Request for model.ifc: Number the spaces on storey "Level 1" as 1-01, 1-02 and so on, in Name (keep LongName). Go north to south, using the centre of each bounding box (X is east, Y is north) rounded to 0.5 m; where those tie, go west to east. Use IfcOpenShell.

First a look at what the model holds.

```python
import ifcopenshell
import ifcopenshell.util.element
import ifcopenshell.util.placement

model = ifcopenshell.open("model.ifc")
print(model.schema)
storey = next(s for s in model.by_type("IfcBuildingStorey") if s.Name == "Level 1")
spaces = [e for e in ifcopenshell.util.element.get_decomposition(storey) if e.is_a("IfcSpace")]
for e in sorted(spaces, key=lambda e: e.id()):
    origin = ifcopenshell.util.placement.get_local_placement(e.ObjectPlacement)[:3, 3]
    print(e.id(), e.Name, e.LongName, origin.round(2) + 0.0, sep=" | ")
```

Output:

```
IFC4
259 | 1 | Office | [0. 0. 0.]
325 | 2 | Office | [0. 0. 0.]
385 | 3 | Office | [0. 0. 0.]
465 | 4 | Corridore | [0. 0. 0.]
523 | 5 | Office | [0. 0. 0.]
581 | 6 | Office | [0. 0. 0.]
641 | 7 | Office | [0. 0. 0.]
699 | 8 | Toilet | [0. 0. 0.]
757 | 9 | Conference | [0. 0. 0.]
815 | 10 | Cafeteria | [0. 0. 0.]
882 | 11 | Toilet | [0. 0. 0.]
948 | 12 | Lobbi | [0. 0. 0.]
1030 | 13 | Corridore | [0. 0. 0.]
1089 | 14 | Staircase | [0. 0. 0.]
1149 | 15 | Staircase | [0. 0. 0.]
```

```python
import ifcopenshell
import ifcopenshell.geom
import ifcopenshell.util.element
import ifcopenshell.util.shape

model = ifcopenshell.open("model.ifc")
settings = ifcopenshell.geom.settings()
settings.set("use-world-coords", True)


def centre(element):
    shape = ifcopenshell.geom.create_shape(settings, element)
    return ifcopenshell.util.shape.get_bbox_centroid(shape.geometry)


storey = next(s for s in model.by_type("IfcBuildingStorey") if s.Name == "Level 1")
spaces = [e for e in ifcopenshell.util.element.get_decomposition(storey) if e.is_a("IfcSpace")]

# Insertion points can sit at a corner or the storey origin, so sort by the geometry (in metres).
centres = {e: centre(e) for e in spaces}
spaces.sort(key=lambda e: (-round(centres[e][1] / 0.5), centres[e][0]))

for i, e in enumerate(spaces, start=1):
    number = f"1-{i:02d}"
    e.Name = number
    print(e.id(), number)

model.write("model_edited.ifc")
```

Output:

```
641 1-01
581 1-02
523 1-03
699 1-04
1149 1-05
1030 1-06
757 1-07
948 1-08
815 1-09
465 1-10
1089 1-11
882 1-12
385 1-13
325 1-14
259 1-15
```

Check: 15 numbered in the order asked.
